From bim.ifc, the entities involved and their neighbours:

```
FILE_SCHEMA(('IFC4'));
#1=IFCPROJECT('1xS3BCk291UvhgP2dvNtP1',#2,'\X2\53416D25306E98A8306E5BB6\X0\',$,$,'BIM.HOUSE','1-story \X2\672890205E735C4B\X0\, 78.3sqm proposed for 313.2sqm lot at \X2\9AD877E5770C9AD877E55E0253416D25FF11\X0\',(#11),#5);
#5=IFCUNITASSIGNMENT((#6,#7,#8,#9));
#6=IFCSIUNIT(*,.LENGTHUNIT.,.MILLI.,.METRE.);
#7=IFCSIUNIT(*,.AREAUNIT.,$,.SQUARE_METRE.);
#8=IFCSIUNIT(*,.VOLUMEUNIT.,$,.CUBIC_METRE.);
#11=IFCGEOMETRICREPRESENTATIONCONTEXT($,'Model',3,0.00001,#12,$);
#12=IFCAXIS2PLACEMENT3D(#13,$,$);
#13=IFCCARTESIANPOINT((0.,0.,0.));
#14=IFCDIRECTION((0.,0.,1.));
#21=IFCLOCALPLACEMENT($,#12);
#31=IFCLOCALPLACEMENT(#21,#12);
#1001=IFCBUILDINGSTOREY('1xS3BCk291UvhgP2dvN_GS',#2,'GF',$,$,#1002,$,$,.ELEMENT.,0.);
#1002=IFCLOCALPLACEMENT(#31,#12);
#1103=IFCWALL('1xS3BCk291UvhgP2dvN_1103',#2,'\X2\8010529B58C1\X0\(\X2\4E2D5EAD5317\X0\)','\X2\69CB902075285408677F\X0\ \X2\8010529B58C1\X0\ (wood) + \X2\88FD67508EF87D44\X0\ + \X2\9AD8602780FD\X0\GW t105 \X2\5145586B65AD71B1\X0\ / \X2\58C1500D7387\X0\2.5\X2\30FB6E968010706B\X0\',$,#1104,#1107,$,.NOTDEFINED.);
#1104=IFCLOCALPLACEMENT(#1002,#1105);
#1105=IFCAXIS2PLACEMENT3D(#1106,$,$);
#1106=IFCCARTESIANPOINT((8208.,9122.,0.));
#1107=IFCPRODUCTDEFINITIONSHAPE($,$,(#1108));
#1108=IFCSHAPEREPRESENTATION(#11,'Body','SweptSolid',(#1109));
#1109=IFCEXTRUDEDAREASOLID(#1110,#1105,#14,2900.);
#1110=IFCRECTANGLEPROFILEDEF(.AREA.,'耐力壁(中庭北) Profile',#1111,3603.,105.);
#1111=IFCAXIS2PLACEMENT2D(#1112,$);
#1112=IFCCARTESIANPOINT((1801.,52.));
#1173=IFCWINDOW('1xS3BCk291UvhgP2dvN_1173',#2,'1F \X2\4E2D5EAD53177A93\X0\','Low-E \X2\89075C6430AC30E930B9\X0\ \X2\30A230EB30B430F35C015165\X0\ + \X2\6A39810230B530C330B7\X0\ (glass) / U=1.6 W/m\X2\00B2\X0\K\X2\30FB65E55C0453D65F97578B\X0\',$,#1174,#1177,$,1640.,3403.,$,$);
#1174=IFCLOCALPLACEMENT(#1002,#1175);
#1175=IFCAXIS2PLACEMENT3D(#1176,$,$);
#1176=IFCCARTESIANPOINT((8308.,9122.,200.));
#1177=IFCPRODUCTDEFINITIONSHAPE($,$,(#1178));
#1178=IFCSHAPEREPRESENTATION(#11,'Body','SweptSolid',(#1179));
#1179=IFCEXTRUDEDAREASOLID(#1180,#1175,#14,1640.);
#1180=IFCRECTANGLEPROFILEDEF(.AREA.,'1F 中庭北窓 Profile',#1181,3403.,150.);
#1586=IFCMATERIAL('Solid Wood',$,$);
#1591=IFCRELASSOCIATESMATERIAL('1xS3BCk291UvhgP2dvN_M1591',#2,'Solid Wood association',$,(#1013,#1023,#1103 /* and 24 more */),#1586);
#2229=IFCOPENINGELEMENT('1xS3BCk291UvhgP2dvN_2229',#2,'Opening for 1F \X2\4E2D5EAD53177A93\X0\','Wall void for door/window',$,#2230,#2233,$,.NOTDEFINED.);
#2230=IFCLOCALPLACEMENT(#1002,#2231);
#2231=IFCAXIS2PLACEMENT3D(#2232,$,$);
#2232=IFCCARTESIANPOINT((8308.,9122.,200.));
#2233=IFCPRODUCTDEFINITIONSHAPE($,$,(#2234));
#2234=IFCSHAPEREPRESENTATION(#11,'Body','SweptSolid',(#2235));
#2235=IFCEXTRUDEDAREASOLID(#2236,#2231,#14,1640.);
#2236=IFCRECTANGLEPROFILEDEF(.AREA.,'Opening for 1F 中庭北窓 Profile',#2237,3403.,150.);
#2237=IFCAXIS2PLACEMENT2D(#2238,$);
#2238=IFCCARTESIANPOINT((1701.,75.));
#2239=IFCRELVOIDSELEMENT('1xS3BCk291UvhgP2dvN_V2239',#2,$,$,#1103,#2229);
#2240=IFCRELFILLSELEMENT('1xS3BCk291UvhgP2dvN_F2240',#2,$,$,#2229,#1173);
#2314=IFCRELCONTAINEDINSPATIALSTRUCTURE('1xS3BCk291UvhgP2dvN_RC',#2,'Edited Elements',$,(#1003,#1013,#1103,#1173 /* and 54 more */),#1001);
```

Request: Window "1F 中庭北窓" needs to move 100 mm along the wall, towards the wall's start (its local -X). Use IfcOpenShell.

```python
import ifcopenshell
import ifcopenshell.api.geometry
import ifcopenshell.util.placement
import ifcopenshell.util.unit

model = ifcopenshell.open("bim.ifc")
unit_scale = ifcopenshell.util.unit.calculate_unit_scale(model)

window = model.by_guid("1xS3BCk291UvhgP2dvN_1173")
opening = window.FillsVoids[0].RelatingOpeningElement
wall = opening.VoidsElements[0].RelatingBuildingElement

wall_matrix = ifcopenshell.util.placement.get_local_placement(wall.ObjectPlacement)
shift = wall_matrix[:3, 0] * -0.1 / unit_scale
before = ifcopenshell.util.placement.get_local_placement(window.ObjectPlacement)[:3, 3].copy()

# The window is not placed relative to its opening, so move both.
for product in (opening, window):
    matrix = ifcopenshell.util.placement.get_local_placement(product.ObjectPlacement)
    matrix[:3, 3] += shift
    ifcopenshell.api.geometry.edit_object_placement(model, product=product, matrix=matrix, is_si=False)

after = ifcopenshell.util.placement.get_local_placement(window.ObjectPlacement)[:3, 3]
print("window moved by", (after - before).round(3) + 0.0)

model.write("bim_v2.ifc")
```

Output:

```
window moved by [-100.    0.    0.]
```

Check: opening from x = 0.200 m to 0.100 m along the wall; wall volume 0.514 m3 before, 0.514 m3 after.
